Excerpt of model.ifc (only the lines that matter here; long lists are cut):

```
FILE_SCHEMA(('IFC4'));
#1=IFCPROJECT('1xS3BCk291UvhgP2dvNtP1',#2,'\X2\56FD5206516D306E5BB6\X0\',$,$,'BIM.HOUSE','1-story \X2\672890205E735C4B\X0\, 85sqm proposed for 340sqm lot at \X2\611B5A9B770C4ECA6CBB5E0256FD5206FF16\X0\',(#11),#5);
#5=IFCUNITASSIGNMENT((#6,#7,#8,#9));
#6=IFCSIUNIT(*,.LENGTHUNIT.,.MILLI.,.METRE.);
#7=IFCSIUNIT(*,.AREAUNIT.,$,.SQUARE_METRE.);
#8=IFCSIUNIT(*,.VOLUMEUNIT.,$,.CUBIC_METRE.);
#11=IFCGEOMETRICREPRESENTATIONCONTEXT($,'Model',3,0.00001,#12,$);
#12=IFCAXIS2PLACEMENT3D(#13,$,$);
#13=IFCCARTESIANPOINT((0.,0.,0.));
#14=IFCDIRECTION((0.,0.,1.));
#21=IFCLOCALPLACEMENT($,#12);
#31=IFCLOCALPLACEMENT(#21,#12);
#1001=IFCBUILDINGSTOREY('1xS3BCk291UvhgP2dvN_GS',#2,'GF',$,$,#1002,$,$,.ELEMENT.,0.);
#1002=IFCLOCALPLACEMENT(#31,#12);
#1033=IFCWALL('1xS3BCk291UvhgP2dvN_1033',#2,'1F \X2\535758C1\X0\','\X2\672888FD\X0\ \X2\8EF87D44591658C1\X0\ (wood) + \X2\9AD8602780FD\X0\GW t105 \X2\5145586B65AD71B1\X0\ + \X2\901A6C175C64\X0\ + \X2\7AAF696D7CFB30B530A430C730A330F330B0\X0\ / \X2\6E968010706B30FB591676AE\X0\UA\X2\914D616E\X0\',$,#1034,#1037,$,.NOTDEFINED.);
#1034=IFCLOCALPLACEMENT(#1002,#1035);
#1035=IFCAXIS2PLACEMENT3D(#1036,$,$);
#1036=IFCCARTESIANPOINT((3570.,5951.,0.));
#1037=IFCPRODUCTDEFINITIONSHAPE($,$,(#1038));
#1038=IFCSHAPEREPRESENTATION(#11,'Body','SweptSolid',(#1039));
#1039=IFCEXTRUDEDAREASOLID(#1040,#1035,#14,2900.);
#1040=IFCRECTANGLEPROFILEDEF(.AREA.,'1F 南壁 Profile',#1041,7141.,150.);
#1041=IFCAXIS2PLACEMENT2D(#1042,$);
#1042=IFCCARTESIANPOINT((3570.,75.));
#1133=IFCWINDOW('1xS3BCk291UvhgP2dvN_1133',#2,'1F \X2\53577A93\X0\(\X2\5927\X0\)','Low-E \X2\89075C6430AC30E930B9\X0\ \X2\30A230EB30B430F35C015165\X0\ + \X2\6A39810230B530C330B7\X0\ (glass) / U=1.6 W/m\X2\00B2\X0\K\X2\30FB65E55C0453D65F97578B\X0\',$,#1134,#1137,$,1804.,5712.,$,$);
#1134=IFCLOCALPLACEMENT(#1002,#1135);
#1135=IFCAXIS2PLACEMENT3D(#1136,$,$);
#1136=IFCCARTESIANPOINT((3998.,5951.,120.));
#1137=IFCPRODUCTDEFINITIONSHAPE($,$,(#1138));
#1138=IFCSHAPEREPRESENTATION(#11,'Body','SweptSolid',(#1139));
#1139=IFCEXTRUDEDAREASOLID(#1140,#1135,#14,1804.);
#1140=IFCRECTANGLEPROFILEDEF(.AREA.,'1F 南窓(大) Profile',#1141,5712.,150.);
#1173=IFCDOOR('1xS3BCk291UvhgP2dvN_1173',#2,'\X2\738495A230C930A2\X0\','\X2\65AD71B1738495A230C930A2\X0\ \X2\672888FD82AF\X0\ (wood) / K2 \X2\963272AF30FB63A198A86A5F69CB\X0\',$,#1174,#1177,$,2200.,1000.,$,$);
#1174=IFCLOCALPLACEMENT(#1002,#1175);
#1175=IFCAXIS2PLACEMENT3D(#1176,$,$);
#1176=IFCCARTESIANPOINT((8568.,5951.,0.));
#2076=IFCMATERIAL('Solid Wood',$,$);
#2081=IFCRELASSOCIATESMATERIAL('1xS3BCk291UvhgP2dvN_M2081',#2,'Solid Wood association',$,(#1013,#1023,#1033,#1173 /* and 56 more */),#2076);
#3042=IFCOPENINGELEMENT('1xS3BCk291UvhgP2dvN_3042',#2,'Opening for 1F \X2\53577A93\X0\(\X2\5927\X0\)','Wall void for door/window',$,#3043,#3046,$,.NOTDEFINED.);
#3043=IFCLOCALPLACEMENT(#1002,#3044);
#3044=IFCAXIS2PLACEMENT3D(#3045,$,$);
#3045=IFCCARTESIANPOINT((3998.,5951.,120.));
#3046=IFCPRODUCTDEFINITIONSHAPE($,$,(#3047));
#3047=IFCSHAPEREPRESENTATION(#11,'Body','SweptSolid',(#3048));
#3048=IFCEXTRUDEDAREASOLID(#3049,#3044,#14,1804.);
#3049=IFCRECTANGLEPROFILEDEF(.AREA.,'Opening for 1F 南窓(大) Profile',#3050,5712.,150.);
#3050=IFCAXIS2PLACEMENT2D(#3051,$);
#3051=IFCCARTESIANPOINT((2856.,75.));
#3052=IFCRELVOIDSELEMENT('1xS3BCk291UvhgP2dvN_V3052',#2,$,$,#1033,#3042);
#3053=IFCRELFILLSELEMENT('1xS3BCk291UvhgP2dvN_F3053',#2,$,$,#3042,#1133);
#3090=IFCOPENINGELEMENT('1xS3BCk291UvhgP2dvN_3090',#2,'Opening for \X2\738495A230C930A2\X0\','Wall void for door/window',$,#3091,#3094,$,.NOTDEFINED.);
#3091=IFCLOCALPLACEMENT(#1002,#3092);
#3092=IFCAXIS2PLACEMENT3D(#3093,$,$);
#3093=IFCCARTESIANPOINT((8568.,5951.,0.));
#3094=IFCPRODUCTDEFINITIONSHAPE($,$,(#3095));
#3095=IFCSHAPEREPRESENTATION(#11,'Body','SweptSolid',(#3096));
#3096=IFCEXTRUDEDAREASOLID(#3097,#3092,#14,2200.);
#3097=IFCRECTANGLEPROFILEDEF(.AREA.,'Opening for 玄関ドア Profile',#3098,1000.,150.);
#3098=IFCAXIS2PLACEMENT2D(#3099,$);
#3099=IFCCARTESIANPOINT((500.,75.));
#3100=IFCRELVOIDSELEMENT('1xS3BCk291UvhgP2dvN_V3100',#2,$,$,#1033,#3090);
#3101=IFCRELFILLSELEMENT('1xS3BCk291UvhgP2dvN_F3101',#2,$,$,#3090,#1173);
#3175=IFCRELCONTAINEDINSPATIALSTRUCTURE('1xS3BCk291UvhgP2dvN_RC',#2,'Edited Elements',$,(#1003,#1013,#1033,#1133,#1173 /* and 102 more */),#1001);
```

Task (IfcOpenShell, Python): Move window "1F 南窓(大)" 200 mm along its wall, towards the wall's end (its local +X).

```python
import ifcopenshell
import ifcopenshell.api.geometry
import ifcopenshell.util.placement
import ifcopenshell.util.unit

model = ifcopenshell.open("model.ifc")
unit_scale = ifcopenshell.util.unit.calculate_unit_scale(model)

window = model.by_guid("1xS3BCk291UvhgP2dvN_1133")
opening = window.FillsVoids[0].RelatingOpeningElement
wall = opening.VoidsElements[0].RelatingBuildingElement

wall_matrix = ifcopenshell.util.placement.get_local_placement(wall.ObjectPlacement)
shift = wall_matrix[:3, 0] * 0.2 / unit_scale
before = ifcopenshell.util.placement.get_local_placement(window.ObjectPlacement)[:3, 3].copy()

# The window is not placed relative to its opening, so move both.
for product in (opening, window):
    matrix = ifcopenshell.util.placement.get_local_placement(product.ObjectPlacement)
    matrix[:3, 3] += shift
    ifcopenshell.api.geometry.edit_object_placement(model, product=product, matrix=matrix, is_si=False)

after = ifcopenshell.util.placement.get_local_placement(window.ObjectPlacement)[:3, 3]
print("window moved by", (after - before).round(3) + 0.0)

model.write("model_edited.ifc")
```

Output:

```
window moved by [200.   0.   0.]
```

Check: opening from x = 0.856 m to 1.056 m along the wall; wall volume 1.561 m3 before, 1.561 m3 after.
